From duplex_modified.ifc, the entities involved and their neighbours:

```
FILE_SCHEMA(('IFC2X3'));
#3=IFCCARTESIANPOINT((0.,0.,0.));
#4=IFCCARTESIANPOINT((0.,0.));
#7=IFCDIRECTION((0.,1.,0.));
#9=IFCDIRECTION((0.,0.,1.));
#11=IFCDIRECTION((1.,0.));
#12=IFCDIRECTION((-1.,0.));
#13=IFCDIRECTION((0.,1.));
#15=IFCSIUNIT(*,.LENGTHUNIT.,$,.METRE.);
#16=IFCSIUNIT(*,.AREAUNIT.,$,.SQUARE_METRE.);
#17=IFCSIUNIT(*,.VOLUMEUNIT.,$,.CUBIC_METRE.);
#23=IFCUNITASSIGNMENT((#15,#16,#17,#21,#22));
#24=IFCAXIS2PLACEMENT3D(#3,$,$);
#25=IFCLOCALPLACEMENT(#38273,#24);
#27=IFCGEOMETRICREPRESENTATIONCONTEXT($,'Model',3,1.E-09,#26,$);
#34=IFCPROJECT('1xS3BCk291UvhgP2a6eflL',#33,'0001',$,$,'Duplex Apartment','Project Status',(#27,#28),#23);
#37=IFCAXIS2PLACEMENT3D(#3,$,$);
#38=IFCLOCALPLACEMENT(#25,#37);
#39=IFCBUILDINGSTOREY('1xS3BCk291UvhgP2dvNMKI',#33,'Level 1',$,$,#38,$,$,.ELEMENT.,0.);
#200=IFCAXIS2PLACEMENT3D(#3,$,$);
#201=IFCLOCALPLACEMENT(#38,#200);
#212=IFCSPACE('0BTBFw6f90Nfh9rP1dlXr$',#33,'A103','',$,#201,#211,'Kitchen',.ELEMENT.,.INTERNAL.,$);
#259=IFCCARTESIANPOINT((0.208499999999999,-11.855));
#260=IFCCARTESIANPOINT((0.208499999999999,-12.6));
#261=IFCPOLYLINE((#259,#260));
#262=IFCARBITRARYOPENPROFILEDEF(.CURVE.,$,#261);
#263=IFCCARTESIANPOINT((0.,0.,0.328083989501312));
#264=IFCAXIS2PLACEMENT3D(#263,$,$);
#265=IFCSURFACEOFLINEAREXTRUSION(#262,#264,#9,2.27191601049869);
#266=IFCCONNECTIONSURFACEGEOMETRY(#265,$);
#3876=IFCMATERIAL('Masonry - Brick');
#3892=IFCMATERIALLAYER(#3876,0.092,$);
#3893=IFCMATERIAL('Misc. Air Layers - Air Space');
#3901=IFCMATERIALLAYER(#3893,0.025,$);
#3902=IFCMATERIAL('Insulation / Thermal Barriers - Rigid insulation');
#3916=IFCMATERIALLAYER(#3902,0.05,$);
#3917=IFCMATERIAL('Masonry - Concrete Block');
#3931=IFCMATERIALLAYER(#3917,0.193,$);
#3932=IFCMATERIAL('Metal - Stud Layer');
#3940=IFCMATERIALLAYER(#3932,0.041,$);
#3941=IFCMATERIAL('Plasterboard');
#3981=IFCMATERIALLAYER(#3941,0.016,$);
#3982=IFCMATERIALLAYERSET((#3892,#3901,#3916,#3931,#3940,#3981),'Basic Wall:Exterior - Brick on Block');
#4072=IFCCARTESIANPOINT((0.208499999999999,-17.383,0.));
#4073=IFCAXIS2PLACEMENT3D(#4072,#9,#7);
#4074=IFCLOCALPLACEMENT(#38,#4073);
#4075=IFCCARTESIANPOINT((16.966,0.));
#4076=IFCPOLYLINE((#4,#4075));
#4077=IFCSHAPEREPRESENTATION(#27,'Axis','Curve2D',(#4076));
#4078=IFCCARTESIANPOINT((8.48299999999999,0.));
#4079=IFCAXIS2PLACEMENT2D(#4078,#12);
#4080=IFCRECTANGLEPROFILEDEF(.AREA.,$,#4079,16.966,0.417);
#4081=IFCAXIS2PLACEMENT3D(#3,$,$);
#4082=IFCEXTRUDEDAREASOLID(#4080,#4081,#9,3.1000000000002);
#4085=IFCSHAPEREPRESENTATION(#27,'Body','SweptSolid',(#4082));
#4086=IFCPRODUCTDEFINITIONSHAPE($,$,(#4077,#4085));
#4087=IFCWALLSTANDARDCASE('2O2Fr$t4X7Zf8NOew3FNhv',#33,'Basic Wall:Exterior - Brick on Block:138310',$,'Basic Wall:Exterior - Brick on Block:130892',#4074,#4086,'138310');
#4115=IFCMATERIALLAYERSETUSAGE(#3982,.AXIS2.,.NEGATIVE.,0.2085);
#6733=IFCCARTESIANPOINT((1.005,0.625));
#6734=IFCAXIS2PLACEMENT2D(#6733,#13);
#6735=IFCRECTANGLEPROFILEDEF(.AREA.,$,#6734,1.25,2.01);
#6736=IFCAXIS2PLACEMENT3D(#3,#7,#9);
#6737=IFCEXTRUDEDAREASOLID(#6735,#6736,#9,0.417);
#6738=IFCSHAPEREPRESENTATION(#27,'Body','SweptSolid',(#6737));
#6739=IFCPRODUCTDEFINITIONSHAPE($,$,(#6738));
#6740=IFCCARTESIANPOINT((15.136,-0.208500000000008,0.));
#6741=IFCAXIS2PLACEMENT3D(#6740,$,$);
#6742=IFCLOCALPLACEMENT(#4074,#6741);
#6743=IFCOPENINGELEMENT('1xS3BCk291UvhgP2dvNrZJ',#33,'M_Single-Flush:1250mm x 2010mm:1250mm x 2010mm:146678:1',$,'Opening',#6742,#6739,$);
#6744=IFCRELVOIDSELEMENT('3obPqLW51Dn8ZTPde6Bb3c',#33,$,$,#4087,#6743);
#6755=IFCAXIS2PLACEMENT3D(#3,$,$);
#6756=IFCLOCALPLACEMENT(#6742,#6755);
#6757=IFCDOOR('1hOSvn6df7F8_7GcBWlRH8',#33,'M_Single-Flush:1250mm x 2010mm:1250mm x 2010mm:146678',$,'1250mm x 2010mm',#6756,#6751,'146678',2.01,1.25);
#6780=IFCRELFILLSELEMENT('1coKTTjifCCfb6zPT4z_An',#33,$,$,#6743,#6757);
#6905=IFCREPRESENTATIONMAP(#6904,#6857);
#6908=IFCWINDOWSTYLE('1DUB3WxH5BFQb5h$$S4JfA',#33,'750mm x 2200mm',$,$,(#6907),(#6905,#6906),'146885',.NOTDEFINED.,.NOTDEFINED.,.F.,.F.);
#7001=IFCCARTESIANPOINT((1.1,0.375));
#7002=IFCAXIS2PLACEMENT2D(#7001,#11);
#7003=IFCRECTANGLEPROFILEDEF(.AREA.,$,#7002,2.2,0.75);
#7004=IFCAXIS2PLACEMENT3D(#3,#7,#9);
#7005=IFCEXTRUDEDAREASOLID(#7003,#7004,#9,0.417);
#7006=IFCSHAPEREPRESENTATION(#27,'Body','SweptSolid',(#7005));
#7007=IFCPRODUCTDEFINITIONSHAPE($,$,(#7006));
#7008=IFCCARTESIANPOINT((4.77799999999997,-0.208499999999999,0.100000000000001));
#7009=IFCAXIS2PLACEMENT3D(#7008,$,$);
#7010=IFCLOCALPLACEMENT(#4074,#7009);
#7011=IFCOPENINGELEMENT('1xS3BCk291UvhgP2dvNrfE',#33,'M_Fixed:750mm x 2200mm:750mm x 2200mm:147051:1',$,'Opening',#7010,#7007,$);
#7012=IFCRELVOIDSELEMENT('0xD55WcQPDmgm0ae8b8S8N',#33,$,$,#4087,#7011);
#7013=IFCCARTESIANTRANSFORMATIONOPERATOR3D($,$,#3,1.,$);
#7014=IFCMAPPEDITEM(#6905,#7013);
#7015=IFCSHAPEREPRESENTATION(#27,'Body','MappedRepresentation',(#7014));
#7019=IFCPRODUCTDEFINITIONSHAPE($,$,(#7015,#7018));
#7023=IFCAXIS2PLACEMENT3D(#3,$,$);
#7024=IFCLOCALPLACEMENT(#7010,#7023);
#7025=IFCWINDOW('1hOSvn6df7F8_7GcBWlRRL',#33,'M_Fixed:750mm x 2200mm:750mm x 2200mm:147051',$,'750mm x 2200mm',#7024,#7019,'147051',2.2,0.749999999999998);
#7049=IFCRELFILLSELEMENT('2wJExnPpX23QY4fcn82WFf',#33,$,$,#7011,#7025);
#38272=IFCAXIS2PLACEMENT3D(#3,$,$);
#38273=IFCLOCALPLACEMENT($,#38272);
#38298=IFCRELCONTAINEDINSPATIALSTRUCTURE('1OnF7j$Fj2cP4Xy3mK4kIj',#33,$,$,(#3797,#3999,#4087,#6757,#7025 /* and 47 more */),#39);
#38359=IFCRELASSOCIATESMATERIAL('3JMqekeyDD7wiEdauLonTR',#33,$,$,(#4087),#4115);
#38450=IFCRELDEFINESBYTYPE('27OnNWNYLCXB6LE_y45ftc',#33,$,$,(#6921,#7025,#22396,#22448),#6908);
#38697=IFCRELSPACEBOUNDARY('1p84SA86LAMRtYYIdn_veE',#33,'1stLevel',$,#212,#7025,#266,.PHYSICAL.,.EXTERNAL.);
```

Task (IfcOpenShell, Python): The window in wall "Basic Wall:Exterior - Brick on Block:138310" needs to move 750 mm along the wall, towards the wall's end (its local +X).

```python
import numpy as np
import ifcopenshell
import ifcopenshell.api.geometry
import ifcopenshell.util.placement

model = ifcopenshell.open("duplex_modified.ifc")

window = model.by_guid("1hOSvn6df7F8_7GcBWlRRL")
opening = window.FillsVoids[0].RelatingOpeningElement
wall = opening.VoidsElements[0].RelatingBuildingElement

wall_matrix = ifcopenshell.util.placement.get_local_placement(wall.ObjectPlacement)
shift = wall_matrix[:3, 0] * 0.75
before = ifcopenshell.util.placement.get_local_placement(window.ObjectPlacement)[:3, 3].copy()

# The window is placed relative to its opening, so it follows when the opening moves.
matrix = ifcopenshell.util.placement.get_local_placement(opening.ObjectPlacement)
matrix[:3, 3] += shift
ifcopenshell.api.geometry.edit_object_placement(
    model, product=opening, matrix=matrix, is_si=False, should_transform_children=True
)

# Space boundary surfaces are stored in each space's coordinates; move them too.
for rel in window.ProvidesBoundaries:
    if not rel.ConnectionGeometry:
        continue
    surface = rel.ConnectionGeometry.SurfaceOnRelatingElement
    space_matrix = ifcopenshell.util.placement.get_local_placement(rel.RelatingSpace.ObjectPlacement)
    point = np.array(surface.Position.Location.Coordinates) + space_matrix[:3, :3].T @ shift
    surface.Position = model.createIfcAxis2Placement3D(
        model.createIfcCartesianPoint(point.tolist()), surface.Position.Axis, surface.Position.RefDirection
    )

after = ifcopenshell.util.placement.get_local_placement(window.ObjectPlacement)[:3, 3]
print("window moved by", (after - before).round(3) + 0.0)

model.write("duplex_modified-out.ifc")
```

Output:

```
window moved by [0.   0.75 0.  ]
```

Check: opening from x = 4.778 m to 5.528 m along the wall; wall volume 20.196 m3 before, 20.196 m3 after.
